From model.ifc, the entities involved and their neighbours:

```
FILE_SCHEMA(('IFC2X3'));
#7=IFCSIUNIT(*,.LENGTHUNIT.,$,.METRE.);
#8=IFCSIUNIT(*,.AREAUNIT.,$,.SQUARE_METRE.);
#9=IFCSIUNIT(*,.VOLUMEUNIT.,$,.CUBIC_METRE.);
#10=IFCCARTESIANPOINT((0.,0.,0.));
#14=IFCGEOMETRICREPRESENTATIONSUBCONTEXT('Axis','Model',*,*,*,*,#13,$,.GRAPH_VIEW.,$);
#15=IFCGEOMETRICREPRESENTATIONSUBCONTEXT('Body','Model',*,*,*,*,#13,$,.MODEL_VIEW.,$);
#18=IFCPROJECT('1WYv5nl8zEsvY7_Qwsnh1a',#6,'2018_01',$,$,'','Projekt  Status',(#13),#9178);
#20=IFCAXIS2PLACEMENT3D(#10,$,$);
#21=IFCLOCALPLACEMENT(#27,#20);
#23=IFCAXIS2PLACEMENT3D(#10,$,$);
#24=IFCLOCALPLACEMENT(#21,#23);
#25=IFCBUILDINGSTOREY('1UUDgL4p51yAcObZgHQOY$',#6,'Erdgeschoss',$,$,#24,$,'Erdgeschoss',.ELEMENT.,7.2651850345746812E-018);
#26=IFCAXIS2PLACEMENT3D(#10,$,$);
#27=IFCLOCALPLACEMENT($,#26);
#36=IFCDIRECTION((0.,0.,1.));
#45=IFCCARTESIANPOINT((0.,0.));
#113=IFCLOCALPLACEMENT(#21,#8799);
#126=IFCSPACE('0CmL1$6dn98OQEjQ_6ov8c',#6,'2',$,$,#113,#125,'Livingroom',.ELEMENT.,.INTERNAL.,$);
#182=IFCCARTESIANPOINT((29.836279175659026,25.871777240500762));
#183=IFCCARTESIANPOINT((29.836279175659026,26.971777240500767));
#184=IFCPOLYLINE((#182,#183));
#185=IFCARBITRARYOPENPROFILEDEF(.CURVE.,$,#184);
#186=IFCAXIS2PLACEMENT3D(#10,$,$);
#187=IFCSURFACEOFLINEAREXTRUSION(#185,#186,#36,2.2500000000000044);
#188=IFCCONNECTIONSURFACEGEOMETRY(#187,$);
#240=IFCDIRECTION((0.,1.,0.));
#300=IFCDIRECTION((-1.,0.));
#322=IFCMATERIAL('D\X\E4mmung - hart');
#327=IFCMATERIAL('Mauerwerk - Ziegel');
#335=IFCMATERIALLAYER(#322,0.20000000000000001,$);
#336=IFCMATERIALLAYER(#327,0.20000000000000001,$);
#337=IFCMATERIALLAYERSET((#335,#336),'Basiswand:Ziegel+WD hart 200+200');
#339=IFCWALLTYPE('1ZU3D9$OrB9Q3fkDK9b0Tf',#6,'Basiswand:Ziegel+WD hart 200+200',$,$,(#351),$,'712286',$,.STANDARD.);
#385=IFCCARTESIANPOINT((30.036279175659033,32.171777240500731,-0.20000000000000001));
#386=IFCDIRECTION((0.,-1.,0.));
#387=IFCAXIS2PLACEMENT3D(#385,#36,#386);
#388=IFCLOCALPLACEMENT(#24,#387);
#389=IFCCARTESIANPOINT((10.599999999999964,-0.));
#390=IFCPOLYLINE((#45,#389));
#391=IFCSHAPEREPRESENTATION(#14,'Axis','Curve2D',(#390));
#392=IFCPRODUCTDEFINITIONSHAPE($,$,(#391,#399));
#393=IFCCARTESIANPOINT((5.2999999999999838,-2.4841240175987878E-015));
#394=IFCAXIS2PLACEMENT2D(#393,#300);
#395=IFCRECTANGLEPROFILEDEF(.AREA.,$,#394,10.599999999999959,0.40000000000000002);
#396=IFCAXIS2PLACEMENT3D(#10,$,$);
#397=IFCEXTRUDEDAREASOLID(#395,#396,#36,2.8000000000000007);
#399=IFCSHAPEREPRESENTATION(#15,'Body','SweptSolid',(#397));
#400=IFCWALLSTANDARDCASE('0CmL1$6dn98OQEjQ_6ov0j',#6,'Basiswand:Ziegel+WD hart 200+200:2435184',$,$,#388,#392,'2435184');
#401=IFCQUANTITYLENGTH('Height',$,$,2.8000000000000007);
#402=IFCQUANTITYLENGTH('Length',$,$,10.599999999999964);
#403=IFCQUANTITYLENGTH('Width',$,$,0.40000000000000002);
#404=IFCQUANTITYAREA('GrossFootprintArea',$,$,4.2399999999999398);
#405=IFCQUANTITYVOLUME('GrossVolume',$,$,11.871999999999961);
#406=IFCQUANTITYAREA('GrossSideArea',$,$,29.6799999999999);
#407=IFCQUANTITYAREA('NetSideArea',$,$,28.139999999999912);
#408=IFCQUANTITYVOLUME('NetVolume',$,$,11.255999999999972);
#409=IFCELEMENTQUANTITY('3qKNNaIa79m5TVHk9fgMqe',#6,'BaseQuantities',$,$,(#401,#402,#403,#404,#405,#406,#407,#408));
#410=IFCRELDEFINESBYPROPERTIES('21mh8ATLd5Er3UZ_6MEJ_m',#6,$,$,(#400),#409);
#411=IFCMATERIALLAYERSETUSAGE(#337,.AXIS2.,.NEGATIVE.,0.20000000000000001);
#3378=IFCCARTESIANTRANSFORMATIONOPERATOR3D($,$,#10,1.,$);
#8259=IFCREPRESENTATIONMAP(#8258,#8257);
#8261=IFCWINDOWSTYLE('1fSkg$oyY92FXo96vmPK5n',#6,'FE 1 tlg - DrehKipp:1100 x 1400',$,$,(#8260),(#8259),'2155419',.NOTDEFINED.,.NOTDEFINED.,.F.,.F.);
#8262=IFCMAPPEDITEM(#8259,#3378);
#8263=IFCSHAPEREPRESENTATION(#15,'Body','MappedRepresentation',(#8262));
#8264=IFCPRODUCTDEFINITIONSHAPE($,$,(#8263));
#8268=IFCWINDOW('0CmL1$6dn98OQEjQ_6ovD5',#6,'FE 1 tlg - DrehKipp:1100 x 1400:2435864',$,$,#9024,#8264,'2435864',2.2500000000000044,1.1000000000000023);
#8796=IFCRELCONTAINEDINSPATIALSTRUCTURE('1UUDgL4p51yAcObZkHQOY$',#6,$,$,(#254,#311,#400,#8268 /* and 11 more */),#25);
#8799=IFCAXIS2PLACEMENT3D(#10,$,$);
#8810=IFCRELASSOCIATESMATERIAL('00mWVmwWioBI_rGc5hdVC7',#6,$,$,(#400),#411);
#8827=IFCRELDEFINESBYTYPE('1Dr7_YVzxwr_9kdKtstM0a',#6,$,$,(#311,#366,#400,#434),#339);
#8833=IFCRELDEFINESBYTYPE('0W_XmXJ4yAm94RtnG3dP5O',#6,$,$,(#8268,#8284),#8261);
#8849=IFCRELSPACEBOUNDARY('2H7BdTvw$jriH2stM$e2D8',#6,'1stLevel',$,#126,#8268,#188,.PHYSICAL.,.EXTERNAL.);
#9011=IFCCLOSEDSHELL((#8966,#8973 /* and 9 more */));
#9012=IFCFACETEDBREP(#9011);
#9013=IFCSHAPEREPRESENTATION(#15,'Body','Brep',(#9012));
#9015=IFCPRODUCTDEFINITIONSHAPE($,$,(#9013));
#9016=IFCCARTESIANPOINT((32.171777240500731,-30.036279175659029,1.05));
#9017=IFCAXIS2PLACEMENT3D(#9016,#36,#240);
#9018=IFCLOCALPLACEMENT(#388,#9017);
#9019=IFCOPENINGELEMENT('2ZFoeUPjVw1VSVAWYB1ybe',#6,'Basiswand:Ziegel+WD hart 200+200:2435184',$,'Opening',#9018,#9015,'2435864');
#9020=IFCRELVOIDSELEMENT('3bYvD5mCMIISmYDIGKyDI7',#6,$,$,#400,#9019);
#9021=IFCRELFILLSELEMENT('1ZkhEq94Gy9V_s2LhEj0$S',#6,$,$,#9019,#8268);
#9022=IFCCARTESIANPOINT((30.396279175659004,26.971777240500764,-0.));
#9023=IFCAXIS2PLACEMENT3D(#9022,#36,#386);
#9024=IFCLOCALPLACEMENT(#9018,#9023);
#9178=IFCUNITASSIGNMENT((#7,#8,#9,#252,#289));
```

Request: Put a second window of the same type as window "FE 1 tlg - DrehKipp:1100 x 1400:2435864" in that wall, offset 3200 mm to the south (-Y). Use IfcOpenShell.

```python
import numpy as np
import ifcopenshell
import ifcopenshell.api.feature
import ifcopenshell.api.geometry
import ifcopenshell.api.pset
import ifcopenshell.api.root
import ifcopenshell.geom
import ifcopenshell.util.element
import ifcopenshell.util.placement
import ifcopenshell.util.shape
import ifcopenshell.util.unit

model = ifcopenshell.open("model.ifc")
unit_scale = ifcopenshell.util.unit.calculate_unit_scale(model)
area_scale = ifcopenshell.util.unit.calculate_unit_scale(model, "AREAUNIT")
volume_scale = ifcopenshell.util.unit.calculate_unit_scale(model, "VOLUMEUNIT")
settings = ifcopenshell.geom.settings()


def volume(element):
    """Net volume in cubic metres, openings subtracted."""
    shape = ifcopenshell.geom.create_shape(settings, element)
    return ifcopenshell.util.shape.get_volume(shape.geometry)


def reuse_history(source, copy):
    """copy_class also copies each property set's owner history, people and application; keep the originals."""
    for rel in copy.IsDefinedBy:
        if rel.is_a("IfcRelDefinesByProperties") and (history := rel.RelatingPropertyDefinition.OwnerHistory):
            rel.RelatingPropertyDefinition.OwnerHistory = source.OwnerHistory
            ifcopenshell.util.element.remove_deep2(model, history)


window = model.by_guid("0CmL1$6dn98OQEjQ_6ovD5")
opening = window.FillsVoids[0].RelatingOpeningElement
wall = opening.VoidsElements[0].RelatingBuildingElement
before = volume(wall)
shift = ifcopenshell.util.placement.get_local_placement(wall.ObjectPlacement)[:3, 0] * 3.2 / unit_scale

# copy_class copies the void relationship, type, container and properties, but no geometry.
new_opening = ifcopenshell.api.root.copy_class(model, product=opening)
new_opening.Representation = ifcopenshell.util.element.copy_deep(
    model, opening.Representation, exclude=["IfcGeometricRepresentationContext", "IfcRepresentationMap"]
)
new_opening.Name = "Basiswand:Ziegel+WD hart 200+200"
new_opening.Tag = None
new_window = ifcopenshell.api.root.copy_class(model, product=window)
new_window.Representation = ifcopenshell.util.element.copy_deep(
    model, window.Representation, exclude=["IfcGeometricRepresentationContext", "IfcRepresentationMap"]
)
new_window.Name = "FE 1 tlg - DrehKipp:1100 x 1400"
new_window.Tag = None
reuse_history(window, new_window)
fills = ifcopenshell.api.feature.add_filling(model, opening=new_opening, element=new_window)
fills.OwnerHistory = new_window.OwnerHistory  # required in IFC2X3

for old, new in ((opening, new_opening), (window, new_window)):
    matrix = ifcopenshell.util.placement.get_local_placement(old.ObjectPlacement)
    matrix[:3, 3] += shift
    ifcopenshell.api.geometry.edit_object_placement(model, product=new, matrix=matrix, is_si=False)

# The copied space boundaries still share their surfaces with the original.
for rel in new_window.ProvidesBoundaries:
    if rel.ConnectionGeometry:
        rel.ConnectionGeometry = ifcopenshell.util.element.copy_deep(model, rel.ConnectionGeometry)

# Space boundary surfaces are stored in each space's coordinates; move them too.
for rel in new_window.ProvidesBoundaries:
    if not rel.ConnectionGeometry:
        continue
    surface = rel.ConnectionGeometry.SurfaceOnRelatingElement
    space_matrix = ifcopenshell.util.placement.get_local_placement(rel.RelatingSpace.ObjectPlacement)
    point = np.array(surface.Position.Location.Coordinates) + space_matrix[:3, :3].T @ shift
    surface.Position = model.createIfcAxis2Placement3D(
        model.createIfcCartesianPoint(point.tolist()), surface.Position.Axis, surface.Position.RefDirection
    )

after = volume(wall)
thickness = 0.4  # wall thickness in metres

# Update the wall's stored quantities.
qto = model.by_id(ifcopenshell.util.element.get_pset(wall, "BaseQuantities", should_inherit=False)["id"])
ifcopenshell.api.pset.edit_qto(model, qto=qto, properties={
    "NetSideArea": after / thickness / area_scale,
    "NetVolume": after / volume_scale,
})

print(f"wall volume {before:.3f} -> {after:.3f} m3")

model.write("model_v2.ifc")
```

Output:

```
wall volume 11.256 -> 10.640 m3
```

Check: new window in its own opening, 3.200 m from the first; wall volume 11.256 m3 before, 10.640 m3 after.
